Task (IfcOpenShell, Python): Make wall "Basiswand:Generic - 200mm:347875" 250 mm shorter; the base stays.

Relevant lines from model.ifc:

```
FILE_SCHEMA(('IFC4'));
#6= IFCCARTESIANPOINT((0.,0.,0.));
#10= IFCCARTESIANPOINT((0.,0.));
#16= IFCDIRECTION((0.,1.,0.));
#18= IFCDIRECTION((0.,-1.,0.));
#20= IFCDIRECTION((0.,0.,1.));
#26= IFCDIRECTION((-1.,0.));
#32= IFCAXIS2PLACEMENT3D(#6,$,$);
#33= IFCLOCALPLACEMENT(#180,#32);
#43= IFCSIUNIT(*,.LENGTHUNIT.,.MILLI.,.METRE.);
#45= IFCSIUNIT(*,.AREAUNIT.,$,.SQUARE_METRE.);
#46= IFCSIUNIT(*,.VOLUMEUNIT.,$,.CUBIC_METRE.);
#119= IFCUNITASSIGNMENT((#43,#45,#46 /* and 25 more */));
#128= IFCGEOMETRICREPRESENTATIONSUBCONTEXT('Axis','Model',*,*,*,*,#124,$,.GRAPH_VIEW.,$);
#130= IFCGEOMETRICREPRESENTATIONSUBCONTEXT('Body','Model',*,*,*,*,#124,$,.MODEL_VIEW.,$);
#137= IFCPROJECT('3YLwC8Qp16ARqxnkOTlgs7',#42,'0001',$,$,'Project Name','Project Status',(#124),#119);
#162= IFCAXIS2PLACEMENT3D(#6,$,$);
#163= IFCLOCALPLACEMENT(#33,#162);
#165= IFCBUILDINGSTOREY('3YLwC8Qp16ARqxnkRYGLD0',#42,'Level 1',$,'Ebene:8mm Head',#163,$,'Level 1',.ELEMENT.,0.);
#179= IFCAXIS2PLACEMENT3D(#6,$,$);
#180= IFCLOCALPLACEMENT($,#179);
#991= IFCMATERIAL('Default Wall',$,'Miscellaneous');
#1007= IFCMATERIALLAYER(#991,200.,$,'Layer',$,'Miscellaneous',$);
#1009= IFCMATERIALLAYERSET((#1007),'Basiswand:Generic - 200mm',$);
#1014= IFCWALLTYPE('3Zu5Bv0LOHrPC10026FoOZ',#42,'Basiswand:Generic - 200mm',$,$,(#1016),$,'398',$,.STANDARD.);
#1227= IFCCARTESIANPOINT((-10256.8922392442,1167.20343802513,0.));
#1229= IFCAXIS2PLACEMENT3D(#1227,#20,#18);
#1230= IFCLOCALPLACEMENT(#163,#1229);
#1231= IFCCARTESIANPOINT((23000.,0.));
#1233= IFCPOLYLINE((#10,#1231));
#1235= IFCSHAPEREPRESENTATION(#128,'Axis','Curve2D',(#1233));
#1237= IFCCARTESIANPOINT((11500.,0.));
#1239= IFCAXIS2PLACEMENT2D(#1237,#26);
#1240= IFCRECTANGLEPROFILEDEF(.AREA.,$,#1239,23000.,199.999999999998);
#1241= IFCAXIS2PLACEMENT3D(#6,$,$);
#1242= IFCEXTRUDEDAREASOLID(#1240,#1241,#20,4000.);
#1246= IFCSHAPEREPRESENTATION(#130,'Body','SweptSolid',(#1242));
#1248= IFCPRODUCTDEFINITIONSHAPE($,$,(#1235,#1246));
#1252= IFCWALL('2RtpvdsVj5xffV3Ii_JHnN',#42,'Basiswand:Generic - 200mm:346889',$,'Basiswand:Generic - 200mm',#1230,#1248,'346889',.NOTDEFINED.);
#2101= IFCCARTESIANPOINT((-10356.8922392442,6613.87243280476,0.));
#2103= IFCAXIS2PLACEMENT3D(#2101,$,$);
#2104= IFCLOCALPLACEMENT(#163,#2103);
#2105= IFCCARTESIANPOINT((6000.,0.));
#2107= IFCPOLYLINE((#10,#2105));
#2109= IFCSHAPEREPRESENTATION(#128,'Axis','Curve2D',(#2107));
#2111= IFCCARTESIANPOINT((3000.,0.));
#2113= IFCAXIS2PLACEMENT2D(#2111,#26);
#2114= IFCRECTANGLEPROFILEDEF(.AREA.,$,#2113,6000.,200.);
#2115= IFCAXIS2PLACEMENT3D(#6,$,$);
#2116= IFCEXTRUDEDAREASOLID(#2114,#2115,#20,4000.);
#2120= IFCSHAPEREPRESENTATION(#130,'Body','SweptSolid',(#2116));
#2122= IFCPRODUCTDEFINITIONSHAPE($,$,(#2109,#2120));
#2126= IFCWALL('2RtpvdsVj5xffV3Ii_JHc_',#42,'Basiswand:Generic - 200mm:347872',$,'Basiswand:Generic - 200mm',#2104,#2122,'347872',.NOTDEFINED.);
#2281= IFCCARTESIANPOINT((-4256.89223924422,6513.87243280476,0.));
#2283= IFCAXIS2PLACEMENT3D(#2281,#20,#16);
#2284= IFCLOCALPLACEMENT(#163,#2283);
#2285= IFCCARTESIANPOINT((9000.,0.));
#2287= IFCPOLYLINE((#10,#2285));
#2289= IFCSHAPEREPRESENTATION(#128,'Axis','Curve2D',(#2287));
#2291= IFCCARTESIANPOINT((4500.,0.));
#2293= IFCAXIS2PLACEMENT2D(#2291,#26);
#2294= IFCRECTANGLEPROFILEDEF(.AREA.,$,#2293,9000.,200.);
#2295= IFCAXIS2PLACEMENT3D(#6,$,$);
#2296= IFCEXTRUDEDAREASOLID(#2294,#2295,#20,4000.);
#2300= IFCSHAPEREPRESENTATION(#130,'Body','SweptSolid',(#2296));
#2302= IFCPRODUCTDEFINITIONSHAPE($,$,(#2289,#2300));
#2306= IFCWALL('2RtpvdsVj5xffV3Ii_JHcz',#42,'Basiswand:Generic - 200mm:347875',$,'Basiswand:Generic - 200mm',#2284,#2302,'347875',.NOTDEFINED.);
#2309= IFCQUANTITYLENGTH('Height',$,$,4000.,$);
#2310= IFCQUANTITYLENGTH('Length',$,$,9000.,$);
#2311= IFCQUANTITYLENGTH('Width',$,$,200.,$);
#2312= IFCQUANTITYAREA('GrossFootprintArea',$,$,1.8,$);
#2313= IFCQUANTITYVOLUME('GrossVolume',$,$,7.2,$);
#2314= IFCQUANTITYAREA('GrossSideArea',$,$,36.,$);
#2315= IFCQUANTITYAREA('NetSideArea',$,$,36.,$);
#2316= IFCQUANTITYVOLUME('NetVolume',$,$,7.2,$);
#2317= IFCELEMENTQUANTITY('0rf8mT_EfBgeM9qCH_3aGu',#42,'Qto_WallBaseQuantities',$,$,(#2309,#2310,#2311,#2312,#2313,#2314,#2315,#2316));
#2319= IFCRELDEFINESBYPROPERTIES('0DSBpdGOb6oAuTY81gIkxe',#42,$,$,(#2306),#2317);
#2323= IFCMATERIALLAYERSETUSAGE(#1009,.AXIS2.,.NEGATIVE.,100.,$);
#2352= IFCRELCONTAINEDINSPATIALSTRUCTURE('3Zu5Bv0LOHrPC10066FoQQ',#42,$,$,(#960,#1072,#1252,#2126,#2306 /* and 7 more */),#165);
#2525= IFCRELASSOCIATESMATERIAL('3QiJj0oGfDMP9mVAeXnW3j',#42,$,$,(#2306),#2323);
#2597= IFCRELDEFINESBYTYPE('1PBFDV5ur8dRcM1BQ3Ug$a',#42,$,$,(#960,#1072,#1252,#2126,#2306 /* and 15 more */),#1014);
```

```python
import ifcopenshell
import ifcopenshell.api.pset
import ifcopenshell.geom
import ifcopenshell.util.element
import ifcopenshell.util.representation
import ifcopenshell.util.shape
import ifcopenshell.util.unit

model = ifcopenshell.open("model.ifc")
unit_scale = ifcopenshell.util.unit.calculate_unit_scale(model)
area_scale = ifcopenshell.util.unit.calculate_unit_scale(model, "AREAUNIT")
volume_scale = ifcopenshell.util.unit.calculate_unit_scale(model, "VOLUMEUNIT")
settings = ifcopenshell.geom.settings()


def volume(element):
    """Net volume in cubic metres, openings subtracted."""
    shape = ifcopenshell.geom.create_shape(settings, element)
    return ifcopenshell.util.shape.get_volume(shape.geometry)


wall = model.by_id(2306)
before = volume(wall)

body = ifcopenshell.util.representation.get_representation(wall, "Model", "Body")
solid = body.Items[0]
old_height = solid.Depth
solid.Depth -= 0.25 / unit_scale
after = volume(wall)
thickness = 0.2  # wall thickness in metres

# Update the stored height, areas and volumes.
qto = model.by_id(ifcopenshell.util.element.get_pset(wall, "Qto_WallBaseQuantities", should_inherit=False)["id"])
ifcopenshell.api.pset.edit_qto(model, qto=qto, properties={
    "Height": solid.Depth,
    "GrossVolume": ifcopenshell.util.element.get_pset(wall, "Qto_WallBaseQuantities", "GrossVolume") * solid.Depth / old_height,
    "GrossSideArea": ifcopenshell.util.element.get_pset(wall, "Qto_WallBaseQuantities", "GrossSideArea") * solid.Depth / old_height,
    "NetSideArea": after / thickness / area_scale,
    "NetVolume": after / volume_scale,
})

print(f"height {old_height:g} -> {solid.Depth:g}, volume {before:.3f} -> {after:.3f} m3")

model.write("model_updated.ifc")
```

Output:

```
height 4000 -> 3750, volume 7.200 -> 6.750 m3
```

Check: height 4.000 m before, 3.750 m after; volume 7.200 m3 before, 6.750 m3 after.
